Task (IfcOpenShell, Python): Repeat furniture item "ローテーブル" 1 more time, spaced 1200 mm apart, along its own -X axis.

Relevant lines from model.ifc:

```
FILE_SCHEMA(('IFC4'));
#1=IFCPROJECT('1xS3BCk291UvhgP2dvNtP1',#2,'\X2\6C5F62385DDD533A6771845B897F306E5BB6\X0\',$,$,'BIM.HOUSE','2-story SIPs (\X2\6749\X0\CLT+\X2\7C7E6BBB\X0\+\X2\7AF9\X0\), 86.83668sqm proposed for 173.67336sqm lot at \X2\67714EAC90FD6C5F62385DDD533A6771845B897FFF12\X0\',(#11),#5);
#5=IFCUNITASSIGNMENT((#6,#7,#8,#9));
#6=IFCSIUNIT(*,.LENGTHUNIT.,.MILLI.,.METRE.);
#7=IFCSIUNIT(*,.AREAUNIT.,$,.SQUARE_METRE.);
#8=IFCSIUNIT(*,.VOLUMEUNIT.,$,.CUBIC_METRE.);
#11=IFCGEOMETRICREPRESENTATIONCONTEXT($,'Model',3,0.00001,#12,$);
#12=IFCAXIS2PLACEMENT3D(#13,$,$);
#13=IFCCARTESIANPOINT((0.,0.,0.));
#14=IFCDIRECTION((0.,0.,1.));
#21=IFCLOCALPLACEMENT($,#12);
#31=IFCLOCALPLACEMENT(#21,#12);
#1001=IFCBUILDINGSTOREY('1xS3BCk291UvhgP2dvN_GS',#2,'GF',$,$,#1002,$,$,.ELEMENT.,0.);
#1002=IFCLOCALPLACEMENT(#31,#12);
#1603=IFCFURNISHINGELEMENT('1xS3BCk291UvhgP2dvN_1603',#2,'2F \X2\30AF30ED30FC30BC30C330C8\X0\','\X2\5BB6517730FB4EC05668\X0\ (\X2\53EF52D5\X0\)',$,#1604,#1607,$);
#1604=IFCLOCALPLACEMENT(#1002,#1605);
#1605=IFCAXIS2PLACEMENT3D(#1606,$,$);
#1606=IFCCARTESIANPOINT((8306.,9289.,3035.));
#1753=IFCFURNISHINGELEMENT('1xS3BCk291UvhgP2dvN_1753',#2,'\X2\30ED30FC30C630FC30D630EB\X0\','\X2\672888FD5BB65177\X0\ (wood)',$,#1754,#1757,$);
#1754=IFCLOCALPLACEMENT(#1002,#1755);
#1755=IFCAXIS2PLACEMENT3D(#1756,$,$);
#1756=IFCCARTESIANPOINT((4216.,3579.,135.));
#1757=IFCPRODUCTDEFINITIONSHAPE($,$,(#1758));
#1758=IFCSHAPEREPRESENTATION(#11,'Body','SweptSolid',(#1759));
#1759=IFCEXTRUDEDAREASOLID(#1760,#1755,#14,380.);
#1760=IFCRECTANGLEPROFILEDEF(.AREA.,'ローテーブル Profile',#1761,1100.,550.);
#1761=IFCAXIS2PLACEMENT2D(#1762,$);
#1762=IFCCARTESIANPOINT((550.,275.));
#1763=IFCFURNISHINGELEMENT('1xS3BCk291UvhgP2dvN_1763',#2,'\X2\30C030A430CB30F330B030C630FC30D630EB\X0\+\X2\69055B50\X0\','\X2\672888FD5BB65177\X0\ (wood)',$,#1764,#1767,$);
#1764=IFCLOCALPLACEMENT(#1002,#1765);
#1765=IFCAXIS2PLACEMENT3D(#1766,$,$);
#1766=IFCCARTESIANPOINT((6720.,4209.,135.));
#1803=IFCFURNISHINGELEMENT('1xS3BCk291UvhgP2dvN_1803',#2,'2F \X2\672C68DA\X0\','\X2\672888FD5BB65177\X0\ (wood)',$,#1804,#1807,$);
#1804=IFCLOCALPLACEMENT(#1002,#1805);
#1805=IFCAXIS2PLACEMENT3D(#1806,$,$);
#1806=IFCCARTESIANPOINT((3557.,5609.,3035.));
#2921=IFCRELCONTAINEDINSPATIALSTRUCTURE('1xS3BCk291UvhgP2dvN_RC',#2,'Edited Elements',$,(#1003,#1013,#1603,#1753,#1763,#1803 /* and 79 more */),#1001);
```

```python
import ifcopenshell
import ifcopenshell.api.geometry
import ifcopenshell.api.root
import ifcopenshell.util.element
import ifcopenshell.util.placement

model = ifcopenshell.open("model.ifc")


def reuse_history(source, copy):
    """copy_class also copies each property set's owner history, people and application; keep the originals."""
    for rel in copy.IsDefinedBy:
        if rel.is_a("IfcRelDefinesByProperties") and (history := rel.RelatingPropertyDefinition.OwnerHistory):
            rel.RelatingPropertyDefinition.OwnerHistory = source.OwnerHistory
            ifcopenshell.util.element.remove_deep2(model, history)


source = model.by_id(1753)
base = ifcopenshell.util.placement.get_local_placement(source.ObjectPlacement)
step = -base[:3, 0] * 1200.0

for i in range(1, 2):
    copy = ifcopenshell.api.root.copy_class(model, product=source)
    copy.Representation = ifcopenshell.util.element.copy_deep(
        model, source.Representation, exclude=["IfcGeometricRepresentationContext", "IfcRepresentationMap"]
    )
    reuse_history(source, copy)
    matrix = base.copy()
    matrix[:3, 3] += i * step
    print("added at", matrix[:3, 3].round(3) + 0.0)
    ifcopenshell.api.geometry.edit_object_placement(model, product=copy, matrix=matrix, is_si=False)

model.write("model_edited.ifc")
```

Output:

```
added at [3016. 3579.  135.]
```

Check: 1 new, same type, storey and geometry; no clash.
